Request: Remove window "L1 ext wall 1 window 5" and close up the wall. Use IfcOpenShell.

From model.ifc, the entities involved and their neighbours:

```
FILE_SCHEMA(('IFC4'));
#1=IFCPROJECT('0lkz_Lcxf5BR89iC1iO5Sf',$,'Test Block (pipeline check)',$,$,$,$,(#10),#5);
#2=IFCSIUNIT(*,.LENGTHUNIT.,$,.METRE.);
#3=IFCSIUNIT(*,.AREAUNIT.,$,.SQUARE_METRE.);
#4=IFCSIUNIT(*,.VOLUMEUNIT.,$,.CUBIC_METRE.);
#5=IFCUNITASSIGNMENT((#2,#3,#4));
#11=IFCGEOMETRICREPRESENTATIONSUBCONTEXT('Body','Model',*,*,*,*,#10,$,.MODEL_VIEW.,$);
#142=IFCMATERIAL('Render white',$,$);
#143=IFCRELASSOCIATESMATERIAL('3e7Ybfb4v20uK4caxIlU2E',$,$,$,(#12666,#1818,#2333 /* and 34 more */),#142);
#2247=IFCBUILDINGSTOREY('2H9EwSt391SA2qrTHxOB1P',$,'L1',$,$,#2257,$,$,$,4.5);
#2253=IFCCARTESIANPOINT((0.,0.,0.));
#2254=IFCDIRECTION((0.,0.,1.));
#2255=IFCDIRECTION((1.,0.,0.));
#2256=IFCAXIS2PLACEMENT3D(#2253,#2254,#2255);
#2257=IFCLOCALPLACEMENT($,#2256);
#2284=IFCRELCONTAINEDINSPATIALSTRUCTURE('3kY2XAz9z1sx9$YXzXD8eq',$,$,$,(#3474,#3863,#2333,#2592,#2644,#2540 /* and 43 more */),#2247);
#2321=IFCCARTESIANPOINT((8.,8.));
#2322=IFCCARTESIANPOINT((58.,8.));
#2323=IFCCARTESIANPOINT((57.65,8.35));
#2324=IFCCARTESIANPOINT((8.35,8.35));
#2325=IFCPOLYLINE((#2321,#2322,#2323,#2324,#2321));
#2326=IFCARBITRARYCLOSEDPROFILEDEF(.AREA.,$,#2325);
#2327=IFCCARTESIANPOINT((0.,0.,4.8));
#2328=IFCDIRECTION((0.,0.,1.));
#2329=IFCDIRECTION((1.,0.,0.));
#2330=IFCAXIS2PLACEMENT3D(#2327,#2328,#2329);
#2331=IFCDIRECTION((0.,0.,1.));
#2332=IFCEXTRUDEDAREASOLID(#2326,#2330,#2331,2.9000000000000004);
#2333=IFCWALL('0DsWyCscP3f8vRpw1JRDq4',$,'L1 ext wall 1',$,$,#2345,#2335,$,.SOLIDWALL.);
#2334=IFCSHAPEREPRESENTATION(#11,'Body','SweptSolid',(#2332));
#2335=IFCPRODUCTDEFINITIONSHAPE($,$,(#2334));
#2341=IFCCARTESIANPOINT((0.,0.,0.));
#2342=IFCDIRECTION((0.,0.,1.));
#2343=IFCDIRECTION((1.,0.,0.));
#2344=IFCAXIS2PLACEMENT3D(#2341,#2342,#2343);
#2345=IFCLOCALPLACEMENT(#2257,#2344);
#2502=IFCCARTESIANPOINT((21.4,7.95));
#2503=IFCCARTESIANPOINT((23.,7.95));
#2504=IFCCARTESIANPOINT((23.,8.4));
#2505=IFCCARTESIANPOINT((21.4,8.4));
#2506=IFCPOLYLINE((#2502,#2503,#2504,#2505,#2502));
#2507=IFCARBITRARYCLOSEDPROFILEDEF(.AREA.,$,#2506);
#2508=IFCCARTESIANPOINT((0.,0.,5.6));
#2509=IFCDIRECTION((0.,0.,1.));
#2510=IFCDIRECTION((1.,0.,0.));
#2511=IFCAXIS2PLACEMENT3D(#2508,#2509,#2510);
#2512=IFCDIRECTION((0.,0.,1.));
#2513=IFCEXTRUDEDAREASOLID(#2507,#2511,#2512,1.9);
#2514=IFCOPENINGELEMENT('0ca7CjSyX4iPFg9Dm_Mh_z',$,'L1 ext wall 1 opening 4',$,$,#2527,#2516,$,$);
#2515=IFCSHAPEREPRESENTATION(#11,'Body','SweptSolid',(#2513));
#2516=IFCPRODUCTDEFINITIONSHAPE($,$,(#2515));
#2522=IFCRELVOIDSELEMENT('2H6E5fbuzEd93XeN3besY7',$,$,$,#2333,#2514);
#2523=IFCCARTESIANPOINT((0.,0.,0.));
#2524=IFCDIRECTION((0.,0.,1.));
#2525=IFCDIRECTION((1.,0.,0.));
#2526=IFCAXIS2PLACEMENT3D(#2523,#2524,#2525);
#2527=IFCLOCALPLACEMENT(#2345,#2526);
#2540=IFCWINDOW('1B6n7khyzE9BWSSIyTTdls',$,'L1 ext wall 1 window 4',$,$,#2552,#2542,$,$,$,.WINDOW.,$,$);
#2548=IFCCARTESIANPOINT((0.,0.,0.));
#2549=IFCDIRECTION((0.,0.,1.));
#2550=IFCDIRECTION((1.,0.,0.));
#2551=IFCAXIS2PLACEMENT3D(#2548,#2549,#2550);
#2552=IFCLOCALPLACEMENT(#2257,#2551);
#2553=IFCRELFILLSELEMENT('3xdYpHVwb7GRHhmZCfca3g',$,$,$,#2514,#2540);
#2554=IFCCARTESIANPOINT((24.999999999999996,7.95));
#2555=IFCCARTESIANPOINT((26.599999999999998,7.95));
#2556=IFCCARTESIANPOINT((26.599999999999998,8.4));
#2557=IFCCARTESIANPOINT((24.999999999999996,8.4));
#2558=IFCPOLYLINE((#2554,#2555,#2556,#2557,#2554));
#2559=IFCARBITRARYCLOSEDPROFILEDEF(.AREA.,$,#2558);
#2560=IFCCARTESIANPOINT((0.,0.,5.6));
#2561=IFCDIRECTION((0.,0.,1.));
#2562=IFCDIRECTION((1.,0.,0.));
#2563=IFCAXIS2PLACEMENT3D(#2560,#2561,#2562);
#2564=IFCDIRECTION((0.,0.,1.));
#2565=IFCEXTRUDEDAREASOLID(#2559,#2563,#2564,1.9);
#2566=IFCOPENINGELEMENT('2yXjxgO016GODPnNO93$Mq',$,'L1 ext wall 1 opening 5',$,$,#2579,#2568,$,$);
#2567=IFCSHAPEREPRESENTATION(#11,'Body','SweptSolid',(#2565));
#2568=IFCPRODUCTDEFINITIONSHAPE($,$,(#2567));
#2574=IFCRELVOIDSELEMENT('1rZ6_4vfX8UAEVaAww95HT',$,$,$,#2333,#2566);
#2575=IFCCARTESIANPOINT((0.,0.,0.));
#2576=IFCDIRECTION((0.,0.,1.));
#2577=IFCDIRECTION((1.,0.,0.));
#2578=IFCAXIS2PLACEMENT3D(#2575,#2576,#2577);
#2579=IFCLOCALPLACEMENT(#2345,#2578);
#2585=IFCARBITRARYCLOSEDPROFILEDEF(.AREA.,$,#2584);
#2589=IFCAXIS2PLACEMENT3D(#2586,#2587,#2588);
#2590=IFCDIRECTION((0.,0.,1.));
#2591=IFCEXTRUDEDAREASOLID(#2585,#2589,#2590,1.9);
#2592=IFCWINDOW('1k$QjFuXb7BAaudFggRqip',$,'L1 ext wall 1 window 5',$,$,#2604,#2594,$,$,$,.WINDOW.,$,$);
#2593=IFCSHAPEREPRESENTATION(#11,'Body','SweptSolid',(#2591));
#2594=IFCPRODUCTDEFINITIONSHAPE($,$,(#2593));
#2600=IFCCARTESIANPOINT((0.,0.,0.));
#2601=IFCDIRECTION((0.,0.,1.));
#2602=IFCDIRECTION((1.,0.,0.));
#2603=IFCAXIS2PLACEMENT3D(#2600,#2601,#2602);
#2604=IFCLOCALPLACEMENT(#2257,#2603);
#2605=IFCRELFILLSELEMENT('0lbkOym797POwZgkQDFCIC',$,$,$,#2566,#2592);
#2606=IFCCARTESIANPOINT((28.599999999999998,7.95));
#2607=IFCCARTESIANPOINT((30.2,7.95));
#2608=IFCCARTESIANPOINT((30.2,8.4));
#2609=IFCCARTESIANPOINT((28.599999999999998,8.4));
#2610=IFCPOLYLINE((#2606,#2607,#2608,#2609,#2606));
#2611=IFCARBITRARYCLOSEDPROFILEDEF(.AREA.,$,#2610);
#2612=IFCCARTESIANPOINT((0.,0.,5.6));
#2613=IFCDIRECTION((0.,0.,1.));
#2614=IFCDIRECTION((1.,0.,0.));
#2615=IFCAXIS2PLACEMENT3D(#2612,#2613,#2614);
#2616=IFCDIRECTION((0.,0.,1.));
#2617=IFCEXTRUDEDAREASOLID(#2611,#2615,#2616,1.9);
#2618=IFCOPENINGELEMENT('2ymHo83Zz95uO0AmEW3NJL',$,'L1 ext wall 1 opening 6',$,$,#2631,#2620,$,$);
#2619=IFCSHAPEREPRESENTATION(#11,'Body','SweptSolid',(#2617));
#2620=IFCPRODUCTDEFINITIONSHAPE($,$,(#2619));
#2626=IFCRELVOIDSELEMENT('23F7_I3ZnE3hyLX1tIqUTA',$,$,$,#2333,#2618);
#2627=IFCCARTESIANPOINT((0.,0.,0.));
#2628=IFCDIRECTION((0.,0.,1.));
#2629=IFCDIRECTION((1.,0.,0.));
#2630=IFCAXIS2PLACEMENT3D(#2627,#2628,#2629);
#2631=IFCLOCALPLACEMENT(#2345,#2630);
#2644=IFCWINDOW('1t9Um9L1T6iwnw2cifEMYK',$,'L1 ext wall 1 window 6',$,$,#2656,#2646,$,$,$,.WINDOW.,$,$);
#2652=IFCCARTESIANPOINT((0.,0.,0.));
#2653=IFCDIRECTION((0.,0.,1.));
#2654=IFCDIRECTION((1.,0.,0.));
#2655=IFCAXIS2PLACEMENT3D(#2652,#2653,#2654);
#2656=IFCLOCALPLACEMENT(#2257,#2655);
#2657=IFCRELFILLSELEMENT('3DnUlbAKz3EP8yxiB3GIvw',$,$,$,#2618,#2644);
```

```python
import ifcopenshell
import ifcopenshell.api.feature
import ifcopenshell.api.root
import ifcopenshell.geom
import ifcopenshell.util.shape

model = ifcopenshell.open("model.ifc")
settings = ifcopenshell.geom.settings()


def volume(element):
    """Net volume in cubic metres, openings subtracted."""
    shape = ifcopenshell.geom.create_shape(settings, element)
    return ifcopenshell.util.shape.get_volume(shape.geometry)


window = model.by_id(2592)
opening = window.FillsVoids[0].RelatingOpeningElement
wall = opening.VoidsElements[0].RelatingBuildingElement
before = volume(wall)

ifcopenshell.api.root.remove_product(model, product=window)
ifcopenshell.api.feature.remove_feature(model, feature=opening)

after = volume(wall)

print(f"wall volume {before:.3f} -> {after:.3f} m3")

model.write("model_edited.ifc")
```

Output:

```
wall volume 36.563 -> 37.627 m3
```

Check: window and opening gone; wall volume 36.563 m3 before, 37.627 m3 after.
